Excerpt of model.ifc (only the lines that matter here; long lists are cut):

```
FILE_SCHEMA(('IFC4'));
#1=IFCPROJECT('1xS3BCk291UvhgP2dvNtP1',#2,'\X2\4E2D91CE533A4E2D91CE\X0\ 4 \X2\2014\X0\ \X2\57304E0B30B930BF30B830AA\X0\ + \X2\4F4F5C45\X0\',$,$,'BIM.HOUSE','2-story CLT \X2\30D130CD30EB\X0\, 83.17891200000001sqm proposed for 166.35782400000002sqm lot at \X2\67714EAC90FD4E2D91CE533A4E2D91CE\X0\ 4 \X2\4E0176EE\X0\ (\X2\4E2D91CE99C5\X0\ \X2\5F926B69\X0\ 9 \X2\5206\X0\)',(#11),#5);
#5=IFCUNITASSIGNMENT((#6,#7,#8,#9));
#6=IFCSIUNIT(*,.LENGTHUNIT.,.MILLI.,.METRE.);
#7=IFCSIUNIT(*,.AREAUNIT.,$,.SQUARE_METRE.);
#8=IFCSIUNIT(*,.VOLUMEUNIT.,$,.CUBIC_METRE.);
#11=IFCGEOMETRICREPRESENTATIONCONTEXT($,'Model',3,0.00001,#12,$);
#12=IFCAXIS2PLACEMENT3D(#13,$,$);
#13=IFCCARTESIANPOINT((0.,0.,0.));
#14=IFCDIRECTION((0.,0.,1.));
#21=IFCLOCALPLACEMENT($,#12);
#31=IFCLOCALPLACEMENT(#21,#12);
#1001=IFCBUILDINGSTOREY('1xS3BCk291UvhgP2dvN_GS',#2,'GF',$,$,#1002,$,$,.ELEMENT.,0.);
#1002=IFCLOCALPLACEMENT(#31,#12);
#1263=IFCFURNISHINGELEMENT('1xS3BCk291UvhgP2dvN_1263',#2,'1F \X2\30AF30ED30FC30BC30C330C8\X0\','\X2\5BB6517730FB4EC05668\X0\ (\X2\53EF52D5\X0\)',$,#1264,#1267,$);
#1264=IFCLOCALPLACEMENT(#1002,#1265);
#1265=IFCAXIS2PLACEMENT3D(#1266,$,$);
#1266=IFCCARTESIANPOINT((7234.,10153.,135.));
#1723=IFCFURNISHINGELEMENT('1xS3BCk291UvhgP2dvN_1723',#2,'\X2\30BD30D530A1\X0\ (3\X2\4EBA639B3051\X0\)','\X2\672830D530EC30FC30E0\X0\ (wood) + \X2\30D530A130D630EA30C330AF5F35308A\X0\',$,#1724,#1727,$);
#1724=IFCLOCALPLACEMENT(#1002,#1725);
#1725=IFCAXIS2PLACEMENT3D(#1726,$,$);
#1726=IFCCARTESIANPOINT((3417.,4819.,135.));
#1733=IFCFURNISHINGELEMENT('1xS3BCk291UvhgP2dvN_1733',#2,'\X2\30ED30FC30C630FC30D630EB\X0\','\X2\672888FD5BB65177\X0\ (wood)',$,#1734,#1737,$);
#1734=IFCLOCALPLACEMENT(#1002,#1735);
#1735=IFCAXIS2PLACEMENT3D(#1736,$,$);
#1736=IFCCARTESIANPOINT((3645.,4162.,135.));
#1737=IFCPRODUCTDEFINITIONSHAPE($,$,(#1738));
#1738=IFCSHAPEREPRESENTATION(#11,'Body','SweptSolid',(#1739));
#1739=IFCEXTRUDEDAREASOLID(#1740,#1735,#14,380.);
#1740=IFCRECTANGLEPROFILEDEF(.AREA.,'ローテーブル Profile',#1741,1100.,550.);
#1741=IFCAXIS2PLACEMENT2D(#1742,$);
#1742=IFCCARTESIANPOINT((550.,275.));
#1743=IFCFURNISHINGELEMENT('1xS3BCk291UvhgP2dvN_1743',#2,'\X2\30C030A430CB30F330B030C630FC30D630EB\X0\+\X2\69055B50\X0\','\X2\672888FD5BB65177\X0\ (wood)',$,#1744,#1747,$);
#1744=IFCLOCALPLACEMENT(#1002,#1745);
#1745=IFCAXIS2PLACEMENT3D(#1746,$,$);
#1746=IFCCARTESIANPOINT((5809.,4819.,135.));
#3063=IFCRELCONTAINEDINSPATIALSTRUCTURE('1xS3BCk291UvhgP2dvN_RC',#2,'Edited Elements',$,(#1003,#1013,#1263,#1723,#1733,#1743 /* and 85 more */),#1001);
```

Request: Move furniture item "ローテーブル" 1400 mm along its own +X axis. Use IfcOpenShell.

```python
import ifcopenshell
import ifcopenshell.api.geometry
import ifcopenshell.util.placement
import ifcopenshell.util.unit

model = ifcopenshell.open("model.ifc")
unit_scale = ifcopenshell.util.unit.calculate_unit_scale(model)

item = model.by_id(1733)
matrix = ifcopenshell.util.placement.get_local_placement(item.ObjectPlacement)
matrix[:3, 3] += matrix[:3, 0] * 1.4 / unit_scale
ifcopenshell.api.geometry.edit_object_placement(model, product=item, matrix=matrix, is_si=False)

print(ifcopenshell.util.placement.get_local_placement(item.ObjectPlacement).round(3) + 0.0)

model.write("model-out.ifc")
```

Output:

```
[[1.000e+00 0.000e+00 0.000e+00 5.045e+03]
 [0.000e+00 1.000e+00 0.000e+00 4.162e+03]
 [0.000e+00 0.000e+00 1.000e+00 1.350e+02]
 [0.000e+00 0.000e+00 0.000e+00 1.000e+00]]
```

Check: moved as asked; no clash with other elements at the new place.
